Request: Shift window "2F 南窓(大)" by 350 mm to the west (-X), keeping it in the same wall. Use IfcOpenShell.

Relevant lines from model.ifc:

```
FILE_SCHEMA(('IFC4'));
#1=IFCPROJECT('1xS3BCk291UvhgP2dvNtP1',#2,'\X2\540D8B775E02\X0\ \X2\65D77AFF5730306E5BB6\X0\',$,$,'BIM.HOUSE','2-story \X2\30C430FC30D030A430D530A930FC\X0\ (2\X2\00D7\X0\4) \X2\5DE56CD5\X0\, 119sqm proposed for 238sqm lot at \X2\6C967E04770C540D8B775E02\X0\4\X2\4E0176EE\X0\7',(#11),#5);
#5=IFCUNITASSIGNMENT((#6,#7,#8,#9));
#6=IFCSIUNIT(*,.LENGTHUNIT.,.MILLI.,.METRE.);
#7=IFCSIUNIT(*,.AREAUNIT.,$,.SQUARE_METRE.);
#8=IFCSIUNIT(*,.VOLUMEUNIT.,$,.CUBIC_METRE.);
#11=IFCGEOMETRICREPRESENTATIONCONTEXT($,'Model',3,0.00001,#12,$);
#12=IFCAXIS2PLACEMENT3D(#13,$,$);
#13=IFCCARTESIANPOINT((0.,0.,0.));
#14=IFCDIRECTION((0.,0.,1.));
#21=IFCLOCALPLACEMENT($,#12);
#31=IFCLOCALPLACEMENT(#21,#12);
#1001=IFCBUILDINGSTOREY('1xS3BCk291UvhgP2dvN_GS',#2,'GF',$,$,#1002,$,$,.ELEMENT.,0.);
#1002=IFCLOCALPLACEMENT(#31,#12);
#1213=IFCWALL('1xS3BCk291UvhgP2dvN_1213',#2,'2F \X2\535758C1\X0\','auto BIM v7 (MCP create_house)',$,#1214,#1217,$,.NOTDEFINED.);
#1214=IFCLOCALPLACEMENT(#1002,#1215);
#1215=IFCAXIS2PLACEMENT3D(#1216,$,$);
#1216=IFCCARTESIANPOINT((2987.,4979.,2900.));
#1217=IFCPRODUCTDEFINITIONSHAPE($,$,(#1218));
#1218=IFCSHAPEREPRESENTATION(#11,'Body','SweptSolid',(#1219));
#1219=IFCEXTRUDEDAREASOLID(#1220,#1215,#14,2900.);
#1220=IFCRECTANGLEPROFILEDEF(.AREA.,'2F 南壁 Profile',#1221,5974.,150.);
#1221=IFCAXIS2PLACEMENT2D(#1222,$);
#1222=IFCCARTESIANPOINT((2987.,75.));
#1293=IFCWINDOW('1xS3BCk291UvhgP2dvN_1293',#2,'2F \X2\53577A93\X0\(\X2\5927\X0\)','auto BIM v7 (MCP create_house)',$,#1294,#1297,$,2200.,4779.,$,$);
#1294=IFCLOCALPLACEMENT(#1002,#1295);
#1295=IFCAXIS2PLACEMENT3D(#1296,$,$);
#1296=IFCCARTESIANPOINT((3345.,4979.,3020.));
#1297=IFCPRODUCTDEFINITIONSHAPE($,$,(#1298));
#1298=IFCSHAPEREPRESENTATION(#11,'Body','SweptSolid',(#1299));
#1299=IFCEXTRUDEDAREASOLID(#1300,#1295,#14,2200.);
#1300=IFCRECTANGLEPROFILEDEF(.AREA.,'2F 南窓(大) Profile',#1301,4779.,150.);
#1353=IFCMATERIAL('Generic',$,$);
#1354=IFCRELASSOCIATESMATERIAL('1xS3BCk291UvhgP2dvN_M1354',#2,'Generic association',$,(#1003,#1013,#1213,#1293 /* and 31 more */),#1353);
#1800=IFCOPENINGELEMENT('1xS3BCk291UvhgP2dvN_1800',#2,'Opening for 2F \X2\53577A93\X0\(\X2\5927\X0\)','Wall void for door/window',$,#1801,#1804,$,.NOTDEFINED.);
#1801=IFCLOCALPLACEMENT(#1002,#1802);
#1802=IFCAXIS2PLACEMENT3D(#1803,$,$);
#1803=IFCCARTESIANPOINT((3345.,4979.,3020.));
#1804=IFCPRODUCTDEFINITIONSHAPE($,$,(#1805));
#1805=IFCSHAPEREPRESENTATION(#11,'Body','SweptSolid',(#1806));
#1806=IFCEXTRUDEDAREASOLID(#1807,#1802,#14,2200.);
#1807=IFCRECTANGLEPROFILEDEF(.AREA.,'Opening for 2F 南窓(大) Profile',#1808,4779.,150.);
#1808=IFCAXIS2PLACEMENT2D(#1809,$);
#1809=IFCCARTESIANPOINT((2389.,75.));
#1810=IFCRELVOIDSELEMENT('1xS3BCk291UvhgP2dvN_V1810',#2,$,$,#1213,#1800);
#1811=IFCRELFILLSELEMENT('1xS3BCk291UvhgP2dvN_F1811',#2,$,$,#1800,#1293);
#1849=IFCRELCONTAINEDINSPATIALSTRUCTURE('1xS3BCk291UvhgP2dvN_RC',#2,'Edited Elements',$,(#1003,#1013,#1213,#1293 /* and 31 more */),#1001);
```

```python
import ifcopenshell
import ifcopenshell.api.geometry
import ifcopenshell.util.placement

model = ifcopenshell.open("model.ifc")

window = model.by_guid("1xS3BCk291UvhgP2dvN_1293")
opening = window.FillsVoids[0].RelatingOpeningElement
wall = opening.VoidsElements[0].RelatingBuildingElement

wall_matrix = ifcopenshell.util.placement.get_local_placement(wall.ObjectPlacement)
shift = wall_matrix[:3, 0] * -350.0
before = ifcopenshell.util.placement.get_local_placement(window.ObjectPlacement)[:3, 3].copy()

# The window is not placed relative to its opening, so move both.
for product in (opening, window):
    matrix = ifcopenshell.util.placement.get_local_placement(product.ObjectPlacement)
    matrix[:3, 3] += shift
    ifcopenshell.api.geometry.edit_object_placement(model, product=product, matrix=matrix, is_si=False)

after = ifcopenshell.util.placement.get_local_placement(window.ObjectPlacement)[:3, 3]
print("window moved by", (after - before).round(3) + 0.0)

model.write("model_edited.ifc")
```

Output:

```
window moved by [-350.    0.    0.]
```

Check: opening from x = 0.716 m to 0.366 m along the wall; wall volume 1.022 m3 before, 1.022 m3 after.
